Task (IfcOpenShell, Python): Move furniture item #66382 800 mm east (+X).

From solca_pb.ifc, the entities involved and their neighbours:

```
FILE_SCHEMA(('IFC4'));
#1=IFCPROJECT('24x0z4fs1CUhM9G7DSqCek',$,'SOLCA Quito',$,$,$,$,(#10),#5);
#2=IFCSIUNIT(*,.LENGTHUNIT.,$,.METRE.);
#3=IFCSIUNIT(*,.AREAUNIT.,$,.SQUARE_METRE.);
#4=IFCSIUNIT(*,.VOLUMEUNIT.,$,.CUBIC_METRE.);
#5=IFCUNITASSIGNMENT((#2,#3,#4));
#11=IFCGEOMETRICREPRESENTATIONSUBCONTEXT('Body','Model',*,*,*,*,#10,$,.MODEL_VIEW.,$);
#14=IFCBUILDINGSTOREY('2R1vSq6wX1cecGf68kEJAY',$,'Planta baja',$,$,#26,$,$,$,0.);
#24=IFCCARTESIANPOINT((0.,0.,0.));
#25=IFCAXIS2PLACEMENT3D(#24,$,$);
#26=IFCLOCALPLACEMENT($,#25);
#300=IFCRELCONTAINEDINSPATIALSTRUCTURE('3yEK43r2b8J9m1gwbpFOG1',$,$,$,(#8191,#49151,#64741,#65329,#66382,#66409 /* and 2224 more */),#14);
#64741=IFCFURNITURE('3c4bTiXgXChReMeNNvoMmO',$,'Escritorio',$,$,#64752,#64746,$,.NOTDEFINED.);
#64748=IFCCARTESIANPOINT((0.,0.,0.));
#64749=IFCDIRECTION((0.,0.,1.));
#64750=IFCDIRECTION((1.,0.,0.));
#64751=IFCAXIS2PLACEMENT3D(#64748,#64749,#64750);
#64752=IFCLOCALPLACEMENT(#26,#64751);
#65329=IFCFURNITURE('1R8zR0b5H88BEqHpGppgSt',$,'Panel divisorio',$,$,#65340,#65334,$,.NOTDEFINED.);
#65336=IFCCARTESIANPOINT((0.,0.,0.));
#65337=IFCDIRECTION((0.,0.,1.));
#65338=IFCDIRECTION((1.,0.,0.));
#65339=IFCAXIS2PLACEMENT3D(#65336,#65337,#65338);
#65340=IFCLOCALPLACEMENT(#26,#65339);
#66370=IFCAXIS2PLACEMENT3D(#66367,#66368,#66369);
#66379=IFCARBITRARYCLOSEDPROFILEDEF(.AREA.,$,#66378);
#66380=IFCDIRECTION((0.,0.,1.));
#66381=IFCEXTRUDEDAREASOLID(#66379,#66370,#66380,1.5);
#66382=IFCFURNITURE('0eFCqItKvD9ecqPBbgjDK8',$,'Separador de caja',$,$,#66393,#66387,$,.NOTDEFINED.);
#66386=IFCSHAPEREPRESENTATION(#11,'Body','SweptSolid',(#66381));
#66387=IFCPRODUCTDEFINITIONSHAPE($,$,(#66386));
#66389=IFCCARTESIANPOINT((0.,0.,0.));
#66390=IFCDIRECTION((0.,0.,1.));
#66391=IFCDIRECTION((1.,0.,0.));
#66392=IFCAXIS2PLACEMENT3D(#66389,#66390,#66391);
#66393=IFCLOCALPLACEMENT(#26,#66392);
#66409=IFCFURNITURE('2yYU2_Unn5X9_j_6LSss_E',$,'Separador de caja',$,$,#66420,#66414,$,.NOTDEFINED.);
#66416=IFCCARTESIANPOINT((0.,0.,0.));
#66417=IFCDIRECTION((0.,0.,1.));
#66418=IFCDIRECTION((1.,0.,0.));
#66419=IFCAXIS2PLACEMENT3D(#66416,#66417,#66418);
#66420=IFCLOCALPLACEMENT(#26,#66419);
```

```python
import ifcopenshell
import ifcopenshell.api.geometry
import ifcopenshell.util.placement
import ifcopenshell.util.unit

model = ifcopenshell.open("solca_pb.ifc")
unit_scale = ifcopenshell.util.unit.calculate_unit_scale(model)

item = model.by_guid("0eFCqItKvD9ecqPBbgjDK8")
matrix = ifcopenshell.util.placement.get_local_placement(item.ObjectPlacement)
matrix[0, 3] += 0.8 / unit_scale
ifcopenshell.api.geometry.edit_object_placement(model, product=item, matrix=matrix, is_si=False)

print(ifcopenshell.util.placement.get_local_placement(item.ObjectPlacement).round(3) + 0.0)

model.write("solca_pb_updated.ifc")
```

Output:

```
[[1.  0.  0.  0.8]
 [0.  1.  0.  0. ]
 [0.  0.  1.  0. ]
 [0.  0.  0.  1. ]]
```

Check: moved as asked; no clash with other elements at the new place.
